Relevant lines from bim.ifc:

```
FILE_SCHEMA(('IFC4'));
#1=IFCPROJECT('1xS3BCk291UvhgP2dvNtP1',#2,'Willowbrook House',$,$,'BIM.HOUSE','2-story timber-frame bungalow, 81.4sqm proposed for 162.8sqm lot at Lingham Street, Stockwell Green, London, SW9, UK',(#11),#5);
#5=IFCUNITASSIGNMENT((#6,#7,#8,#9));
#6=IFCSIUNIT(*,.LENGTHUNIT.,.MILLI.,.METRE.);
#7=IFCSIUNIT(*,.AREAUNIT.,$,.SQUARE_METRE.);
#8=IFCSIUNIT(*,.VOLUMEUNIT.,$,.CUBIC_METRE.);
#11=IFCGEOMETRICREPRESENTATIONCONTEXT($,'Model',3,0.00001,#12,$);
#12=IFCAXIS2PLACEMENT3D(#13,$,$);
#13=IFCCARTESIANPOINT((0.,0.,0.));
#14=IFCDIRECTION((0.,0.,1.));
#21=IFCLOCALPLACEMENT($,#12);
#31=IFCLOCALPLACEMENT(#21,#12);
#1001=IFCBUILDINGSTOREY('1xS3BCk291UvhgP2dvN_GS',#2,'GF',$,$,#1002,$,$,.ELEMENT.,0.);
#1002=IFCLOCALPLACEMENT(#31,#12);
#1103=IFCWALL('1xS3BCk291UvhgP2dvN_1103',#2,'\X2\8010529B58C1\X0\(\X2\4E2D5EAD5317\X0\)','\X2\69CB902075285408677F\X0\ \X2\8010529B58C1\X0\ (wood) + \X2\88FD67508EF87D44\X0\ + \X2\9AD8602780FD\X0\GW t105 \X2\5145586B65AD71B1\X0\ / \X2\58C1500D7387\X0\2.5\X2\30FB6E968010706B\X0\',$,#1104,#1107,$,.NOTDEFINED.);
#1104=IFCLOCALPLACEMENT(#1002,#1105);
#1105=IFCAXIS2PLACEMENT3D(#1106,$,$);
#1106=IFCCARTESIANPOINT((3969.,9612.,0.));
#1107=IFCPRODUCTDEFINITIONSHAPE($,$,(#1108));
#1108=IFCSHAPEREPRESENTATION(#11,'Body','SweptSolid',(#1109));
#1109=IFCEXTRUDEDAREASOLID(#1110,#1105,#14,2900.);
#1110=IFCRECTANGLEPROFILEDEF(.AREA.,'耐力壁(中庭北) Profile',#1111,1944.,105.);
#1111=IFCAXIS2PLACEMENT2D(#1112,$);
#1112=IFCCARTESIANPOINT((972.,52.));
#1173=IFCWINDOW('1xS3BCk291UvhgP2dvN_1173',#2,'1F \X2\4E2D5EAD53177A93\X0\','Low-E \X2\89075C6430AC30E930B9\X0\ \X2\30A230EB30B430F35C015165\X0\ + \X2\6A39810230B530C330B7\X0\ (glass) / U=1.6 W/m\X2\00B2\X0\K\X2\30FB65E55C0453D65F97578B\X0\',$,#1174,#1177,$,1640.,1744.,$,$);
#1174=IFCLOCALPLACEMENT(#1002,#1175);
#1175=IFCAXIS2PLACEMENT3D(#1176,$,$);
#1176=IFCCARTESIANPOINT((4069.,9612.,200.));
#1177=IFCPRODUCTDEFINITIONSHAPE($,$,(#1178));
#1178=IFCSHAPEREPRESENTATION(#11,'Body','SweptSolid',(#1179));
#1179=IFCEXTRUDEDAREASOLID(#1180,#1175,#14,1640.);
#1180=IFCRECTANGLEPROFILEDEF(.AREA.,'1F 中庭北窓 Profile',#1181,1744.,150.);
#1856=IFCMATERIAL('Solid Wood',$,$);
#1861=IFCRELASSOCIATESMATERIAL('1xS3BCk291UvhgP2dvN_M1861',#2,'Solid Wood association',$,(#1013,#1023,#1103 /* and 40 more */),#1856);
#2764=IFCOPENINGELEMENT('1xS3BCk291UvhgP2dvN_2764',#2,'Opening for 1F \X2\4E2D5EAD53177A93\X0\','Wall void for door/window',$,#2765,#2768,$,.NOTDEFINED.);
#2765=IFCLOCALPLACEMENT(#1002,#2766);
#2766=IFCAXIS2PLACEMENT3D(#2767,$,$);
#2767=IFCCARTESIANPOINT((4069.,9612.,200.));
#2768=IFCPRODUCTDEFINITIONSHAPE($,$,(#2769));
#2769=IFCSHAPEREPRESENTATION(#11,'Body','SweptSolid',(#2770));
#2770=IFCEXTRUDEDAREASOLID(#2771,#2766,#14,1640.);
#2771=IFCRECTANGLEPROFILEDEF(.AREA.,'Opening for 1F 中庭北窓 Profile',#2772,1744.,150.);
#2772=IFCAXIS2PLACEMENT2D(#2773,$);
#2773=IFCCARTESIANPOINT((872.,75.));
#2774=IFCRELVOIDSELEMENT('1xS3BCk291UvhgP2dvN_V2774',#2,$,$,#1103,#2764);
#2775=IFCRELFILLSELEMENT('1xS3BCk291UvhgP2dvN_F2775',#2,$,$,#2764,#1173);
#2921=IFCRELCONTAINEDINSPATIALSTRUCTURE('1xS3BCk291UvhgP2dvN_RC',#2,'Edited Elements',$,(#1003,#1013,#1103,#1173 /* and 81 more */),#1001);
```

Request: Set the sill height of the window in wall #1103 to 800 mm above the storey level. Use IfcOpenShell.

```python
import numpy as np
import ifcopenshell
import ifcopenshell.api.geometry
import ifcopenshell.geom
import ifcopenshell.util.element
import ifcopenshell.util.placement
import ifcopenshell.util.shape
import ifcopenshell.util.unit

model = ifcopenshell.open("bim.ifc")
unit_scale = ifcopenshell.util.unit.calculate_unit_scale(model)

window = model.by_guid("1xS3BCk291UvhgP2dvN_1173")
opening = window.FillsVoids[0].RelatingOpeningElement
storey = ifcopenshell.util.element.get_container(window, ifc_class="IfcBuildingStorey")
level = ifcopenshell.util.placement.get_local_placement(storey.ObjectPlacement)[2, 3]

# The opening's origin need not be at the sill, so measure its lowest point.
shape = ifcopenshell.geom.create_shape(ifcopenshell.geom.settings(), opening)
bottom = ifcopenshell.util.shape.get_shape_bottom_elevation(shape, shape.geometry) / unit_scale
dz = level + 0.8 / unit_scale - bottom

shift = np.array([0.0, 0.0, dz])
# The window is not placed relative to its opening, so move both.
for product in (opening, window):
    matrix = ifcopenshell.util.placement.get_local_placement(product.ObjectPlacement)
    matrix[:3, 3] += shift
    ifcopenshell.api.geometry.edit_object_placement(model, product=product, matrix=matrix, is_si=False)

print(f"moved by {dz * unit_scale:+.3f} m")

model.write("bim_v2.ifc")
```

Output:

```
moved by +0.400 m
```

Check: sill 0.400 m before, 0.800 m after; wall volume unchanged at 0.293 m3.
